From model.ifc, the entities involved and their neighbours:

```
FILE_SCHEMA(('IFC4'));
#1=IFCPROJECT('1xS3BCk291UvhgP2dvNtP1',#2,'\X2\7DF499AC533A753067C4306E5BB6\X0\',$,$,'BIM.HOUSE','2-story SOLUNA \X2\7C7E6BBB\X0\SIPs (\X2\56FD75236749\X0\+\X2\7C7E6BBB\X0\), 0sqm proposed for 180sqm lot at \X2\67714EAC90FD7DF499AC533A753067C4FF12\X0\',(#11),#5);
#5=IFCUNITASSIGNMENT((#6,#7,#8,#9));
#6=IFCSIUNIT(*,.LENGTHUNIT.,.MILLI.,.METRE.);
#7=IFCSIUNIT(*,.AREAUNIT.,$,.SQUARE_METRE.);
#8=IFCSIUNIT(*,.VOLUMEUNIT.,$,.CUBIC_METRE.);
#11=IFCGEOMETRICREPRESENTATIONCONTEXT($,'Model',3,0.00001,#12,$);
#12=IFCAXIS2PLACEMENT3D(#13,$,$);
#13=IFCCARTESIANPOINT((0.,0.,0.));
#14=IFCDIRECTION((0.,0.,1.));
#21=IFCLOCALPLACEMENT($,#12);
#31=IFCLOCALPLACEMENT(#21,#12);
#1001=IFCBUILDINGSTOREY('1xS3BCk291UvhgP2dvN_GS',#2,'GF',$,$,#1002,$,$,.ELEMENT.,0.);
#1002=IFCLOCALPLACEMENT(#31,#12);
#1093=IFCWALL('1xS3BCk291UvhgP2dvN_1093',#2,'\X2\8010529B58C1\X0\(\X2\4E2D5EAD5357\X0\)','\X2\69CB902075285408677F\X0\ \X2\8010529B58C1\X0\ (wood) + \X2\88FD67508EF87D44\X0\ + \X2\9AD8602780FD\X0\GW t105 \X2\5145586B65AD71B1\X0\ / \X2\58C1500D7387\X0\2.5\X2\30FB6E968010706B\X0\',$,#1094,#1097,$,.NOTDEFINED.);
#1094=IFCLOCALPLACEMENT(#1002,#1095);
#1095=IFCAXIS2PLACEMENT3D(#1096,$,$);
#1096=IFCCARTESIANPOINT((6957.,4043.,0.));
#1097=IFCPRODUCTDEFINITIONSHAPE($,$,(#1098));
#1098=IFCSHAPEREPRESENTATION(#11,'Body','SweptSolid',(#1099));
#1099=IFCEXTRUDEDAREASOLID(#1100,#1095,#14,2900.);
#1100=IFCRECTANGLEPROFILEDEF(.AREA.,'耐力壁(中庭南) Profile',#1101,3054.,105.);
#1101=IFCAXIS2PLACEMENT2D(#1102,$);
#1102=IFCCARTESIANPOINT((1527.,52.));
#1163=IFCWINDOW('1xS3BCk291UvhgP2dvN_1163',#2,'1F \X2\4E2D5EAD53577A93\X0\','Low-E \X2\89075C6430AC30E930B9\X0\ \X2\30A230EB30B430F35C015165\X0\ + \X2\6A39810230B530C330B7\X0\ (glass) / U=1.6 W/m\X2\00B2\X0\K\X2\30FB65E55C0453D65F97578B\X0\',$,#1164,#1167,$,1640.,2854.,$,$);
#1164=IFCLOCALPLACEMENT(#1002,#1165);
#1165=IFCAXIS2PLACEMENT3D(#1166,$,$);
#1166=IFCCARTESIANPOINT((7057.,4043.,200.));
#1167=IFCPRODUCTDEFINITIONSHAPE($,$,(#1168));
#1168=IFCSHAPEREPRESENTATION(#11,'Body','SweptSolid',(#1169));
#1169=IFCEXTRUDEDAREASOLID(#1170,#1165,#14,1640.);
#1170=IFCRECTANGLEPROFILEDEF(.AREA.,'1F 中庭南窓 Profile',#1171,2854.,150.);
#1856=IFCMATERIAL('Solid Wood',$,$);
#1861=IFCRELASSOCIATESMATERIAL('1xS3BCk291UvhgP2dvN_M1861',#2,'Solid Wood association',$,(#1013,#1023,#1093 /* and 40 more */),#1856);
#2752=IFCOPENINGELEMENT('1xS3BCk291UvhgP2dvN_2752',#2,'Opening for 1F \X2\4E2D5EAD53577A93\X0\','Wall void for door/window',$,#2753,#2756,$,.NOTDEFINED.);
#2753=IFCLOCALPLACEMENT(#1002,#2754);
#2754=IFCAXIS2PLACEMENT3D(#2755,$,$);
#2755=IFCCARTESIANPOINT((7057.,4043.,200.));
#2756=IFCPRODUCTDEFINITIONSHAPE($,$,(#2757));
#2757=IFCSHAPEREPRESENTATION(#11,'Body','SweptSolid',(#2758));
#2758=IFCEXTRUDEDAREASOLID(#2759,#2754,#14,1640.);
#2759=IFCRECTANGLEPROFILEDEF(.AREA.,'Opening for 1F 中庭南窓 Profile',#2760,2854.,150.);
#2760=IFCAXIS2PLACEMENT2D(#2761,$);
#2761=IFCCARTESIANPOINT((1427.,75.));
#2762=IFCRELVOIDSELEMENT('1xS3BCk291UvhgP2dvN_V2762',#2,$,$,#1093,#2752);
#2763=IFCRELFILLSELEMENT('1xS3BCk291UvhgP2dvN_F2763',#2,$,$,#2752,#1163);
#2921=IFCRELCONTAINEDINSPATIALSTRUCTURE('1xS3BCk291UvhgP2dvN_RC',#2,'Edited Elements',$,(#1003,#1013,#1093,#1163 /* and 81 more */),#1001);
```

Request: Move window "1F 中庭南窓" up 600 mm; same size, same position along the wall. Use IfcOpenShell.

```python
import numpy as np
import ifcopenshell
import ifcopenshell.api.geometry
import ifcopenshell.util.placement
import ifcopenshell.util.unit

model = ifcopenshell.open("model.ifc")
unit_scale = ifcopenshell.util.unit.calculate_unit_scale(model)

window = model.by_id(1163)
opening = window.FillsVoids[0].RelatingOpeningElement
dz = 0.6 / unit_scale

shift = np.array([0.0, 0.0, dz])
# The window is not placed relative to its opening, so move both.
for product in (opening, window):
    matrix = ifcopenshell.util.placement.get_local_placement(product.ObjectPlacement)
    matrix[:3, 3] += shift
    ifcopenshell.api.geometry.edit_object_placement(model, product=product, matrix=matrix, is_si=False)

print(f"moved by {dz * unit_scale:+.3f} m")

model.write("model_updated.ifc")
```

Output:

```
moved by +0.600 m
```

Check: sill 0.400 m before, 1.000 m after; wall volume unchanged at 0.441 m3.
